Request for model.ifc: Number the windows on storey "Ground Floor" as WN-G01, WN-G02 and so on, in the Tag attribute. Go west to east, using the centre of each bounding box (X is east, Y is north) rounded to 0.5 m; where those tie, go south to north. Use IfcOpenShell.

First a look at what the model holds.

```python
import ifcopenshell
import ifcopenshell.util.element
import ifcopenshell.util.placement

model = ifcopenshell.open("model.ifc")
print(model.schema)
storey = next(s for s in model.by_type("IfcBuildingStorey") if s.Name == "Ground Floor")
windows = [e for e in ifcopenshell.util.element.get_decomposition(storey) if e.is_a("IfcWindow")]
for e in sorted(windows, key=lambda e: e.id()):
    origin = ifcopenshell.util.placement.get_local_placement(e.ObjectPlacement)[:3, 3]
    print(e.id(), e.Tag, e.Name, origin.round(2) + 0.0, sep=" | ")
```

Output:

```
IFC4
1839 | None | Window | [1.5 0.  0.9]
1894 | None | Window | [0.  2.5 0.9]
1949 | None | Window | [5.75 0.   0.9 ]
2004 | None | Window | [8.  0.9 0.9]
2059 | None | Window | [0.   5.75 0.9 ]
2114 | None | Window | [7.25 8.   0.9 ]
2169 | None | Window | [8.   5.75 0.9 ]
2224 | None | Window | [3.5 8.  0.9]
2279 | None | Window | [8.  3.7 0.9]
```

```python
import ifcopenshell
import ifcopenshell.geom
import ifcopenshell.util.element
import ifcopenshell.util.shape

model = ifcopenshell.open("model.ifc")
settings = ifcopenshell.geom.settings()
settings.set("use-world-coords", True)


def centre(element):
    shape = ifcopenshell.geom.create_shape(settings, element)
    return ifcopenshell.util.shape.get_bbox_centroid(shape.geometry)


storey = next(s for s in model.by_type("IfcBuildingStorey") if s.Name == "Ground Floor")
windows = [e for e in ifcopenshell.util.element.get_decomposition(storey) if e.is_a("IfcWindow")]

# Insertion points can sit at a corner or the storey origin, so sort by the geometry (in metres).
centres = {e: centre(e) for e in windows}
windows.sort(key=lambda e: (round(centres[e][0] / 0.5), centres[e][1]))

for i, e in enumerate(windows, start=1):
    number = f"WN-G{i:02d}"
    e.Tag = number
    print(e.id(), number)

model.write("model-out.ifc")
```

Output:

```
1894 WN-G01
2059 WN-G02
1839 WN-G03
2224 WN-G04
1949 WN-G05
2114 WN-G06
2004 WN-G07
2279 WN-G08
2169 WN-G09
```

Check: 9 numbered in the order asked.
